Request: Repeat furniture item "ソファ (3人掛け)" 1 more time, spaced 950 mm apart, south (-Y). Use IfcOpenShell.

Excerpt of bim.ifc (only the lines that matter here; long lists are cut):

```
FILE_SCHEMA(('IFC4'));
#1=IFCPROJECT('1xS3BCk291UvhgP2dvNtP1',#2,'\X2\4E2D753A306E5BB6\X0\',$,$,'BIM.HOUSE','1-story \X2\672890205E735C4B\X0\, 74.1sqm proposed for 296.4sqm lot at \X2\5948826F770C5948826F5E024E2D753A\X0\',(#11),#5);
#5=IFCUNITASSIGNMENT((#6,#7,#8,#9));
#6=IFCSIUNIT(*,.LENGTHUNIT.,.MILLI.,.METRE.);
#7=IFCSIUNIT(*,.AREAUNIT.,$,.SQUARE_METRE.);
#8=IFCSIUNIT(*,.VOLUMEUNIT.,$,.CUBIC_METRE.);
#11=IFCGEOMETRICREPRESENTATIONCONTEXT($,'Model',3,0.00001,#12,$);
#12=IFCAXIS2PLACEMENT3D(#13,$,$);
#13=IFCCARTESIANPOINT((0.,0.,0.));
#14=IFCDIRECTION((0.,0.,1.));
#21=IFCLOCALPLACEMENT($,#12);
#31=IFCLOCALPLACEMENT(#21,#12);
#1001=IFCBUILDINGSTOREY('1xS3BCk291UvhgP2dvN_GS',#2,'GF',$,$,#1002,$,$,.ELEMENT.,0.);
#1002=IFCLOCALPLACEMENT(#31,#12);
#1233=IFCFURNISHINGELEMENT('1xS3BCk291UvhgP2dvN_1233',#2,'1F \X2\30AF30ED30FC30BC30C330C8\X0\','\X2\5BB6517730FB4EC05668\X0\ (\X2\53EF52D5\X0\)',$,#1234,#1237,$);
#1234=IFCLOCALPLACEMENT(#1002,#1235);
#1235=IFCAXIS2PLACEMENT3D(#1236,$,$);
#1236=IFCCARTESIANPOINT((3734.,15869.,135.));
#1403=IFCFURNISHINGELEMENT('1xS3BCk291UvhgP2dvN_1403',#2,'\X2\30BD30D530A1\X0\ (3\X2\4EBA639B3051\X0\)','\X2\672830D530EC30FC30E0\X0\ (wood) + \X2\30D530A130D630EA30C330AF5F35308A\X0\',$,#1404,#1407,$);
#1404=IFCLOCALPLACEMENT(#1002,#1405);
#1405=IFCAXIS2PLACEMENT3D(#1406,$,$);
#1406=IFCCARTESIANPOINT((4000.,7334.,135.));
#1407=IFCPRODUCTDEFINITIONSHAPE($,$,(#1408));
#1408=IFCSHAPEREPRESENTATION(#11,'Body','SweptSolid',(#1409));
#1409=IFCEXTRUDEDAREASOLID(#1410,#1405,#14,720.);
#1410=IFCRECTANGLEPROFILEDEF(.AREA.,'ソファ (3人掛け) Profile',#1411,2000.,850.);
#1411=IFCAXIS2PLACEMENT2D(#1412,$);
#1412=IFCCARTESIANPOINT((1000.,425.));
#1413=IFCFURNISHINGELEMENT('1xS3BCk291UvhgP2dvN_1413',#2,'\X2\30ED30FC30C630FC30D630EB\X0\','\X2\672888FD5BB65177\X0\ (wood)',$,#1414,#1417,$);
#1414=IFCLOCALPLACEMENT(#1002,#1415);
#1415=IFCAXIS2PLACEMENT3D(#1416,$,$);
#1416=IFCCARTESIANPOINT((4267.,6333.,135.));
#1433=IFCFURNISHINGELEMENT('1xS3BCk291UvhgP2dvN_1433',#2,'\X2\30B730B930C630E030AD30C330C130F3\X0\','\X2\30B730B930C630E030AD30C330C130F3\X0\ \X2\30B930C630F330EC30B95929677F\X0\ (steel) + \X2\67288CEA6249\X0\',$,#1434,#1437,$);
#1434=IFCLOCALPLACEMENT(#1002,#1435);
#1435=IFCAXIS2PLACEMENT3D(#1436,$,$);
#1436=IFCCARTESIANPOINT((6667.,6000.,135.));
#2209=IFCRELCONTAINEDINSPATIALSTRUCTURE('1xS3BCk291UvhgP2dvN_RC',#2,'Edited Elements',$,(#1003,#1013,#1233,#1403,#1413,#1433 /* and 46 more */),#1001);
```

```python
import numpy as np
import ifcopenshell
import ifcopenshell.api.geometry
import ifcopenshell.api.root
import ifcopenshell.util.element
import ifcopenshell.util.placement

model = ifcopenshell.open("bim.ifc")


def reuse_history(source, copy):
    """copy_class also copies each property set's owner history, people and application; keep the originals."""
    for rel in copy.IsDefinedBy:
        if rel.is_a("IfcRelDefinesByProperties") and (history := rel.RelatingPropertyDefinition.OwnerHistory):
            rel.RelatingPropertyDefinition.OwnerHistory = source.OwnerHistory
            ifcopenshell.util.element.remove_deep2(model, history)


source = model.by_guid("1xS3BCk291UvhgP2dvN_1403")
base = ifcopenshell.util.placement.get_local_placement(source.ObjectPlacement)
step = np.array([0.0, -1.0, 0.0]) * 950.0

for i in range(1, 2):
    copy = ifcopenshell.api.root.copy_class(model, product=source)
    copy.Representation = ifcopenshell.util.element.copy_deep(
        model, source.Representation, exclude=["IfcGeometricRepresentationContext", "IfcRepresentationMap"]
    )
    reuse_history(source, copy)
    matrix = base.copy()
    matrix[:3, 3] += i * step
    print("added at", matrix[:3, 3].round(3) + 0.0)
    ifcopenshell.api.geometry.edit_object_placement(model, product=copy, matrix=matrix, is_si=False)

model.write("bim-out.ifc")
```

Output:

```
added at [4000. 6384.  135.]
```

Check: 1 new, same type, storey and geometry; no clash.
